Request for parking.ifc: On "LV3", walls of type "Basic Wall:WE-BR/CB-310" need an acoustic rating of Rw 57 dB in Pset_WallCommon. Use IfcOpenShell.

First a look at what the model holds.

```python
import ifcopenshell
import ifcopenshell.util.element

model = ifcopenshell.open("parking.ifc")
print(model.schema)
storey = next(s for s in model.by_type("IfcBuildingStorey") if s.Name == "LV3")
walls = [e for e in ifcopenshell.util.element.get_decomposition(storey) if e.is_a("IfcWall")]
seen = {}
for e in walls:
    element_type = ifcopenshell.util.element.get_type(e)
    key = (element_type.Name if element_type != e and element_type else None, ifcopenshell.util.element.get_pset(e, "Pset_WallCommon", "AcousticRating"))
    seen[key] = seen.get(key, 0) + 1
for (name, value), count in sorted(seen.items(), key=str):
    print(count, "x", name, "|", value)
```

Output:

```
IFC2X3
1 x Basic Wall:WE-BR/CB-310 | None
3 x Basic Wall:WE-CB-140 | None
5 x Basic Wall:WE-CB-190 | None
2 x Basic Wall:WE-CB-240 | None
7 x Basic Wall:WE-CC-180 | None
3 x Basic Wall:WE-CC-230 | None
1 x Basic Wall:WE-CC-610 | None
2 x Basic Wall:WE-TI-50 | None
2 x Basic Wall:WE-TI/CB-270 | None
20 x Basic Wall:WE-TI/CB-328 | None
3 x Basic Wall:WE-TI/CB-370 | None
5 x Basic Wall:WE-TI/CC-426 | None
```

```python
import ifcopenshell
import ifcopenshell.api.pset
import ifcopenshell.util.element

model = ifcopenshell.open("parking.ifc")

storey = next(s for s in model.by_type("IfcBuildingStorey") if s.Name == "LV3")
walls = [e for e in ifcopenshell.util.element.get_decomposition(storey) if e.is_a("IfcWall")]

count = 0
for e in walls:
    element_type = ifcopenshell.util.element.get_type(e)
    if element_type in (None, e) or element_type.Name != "Basic Wall:WE-BR/CB-310":
        continue
    # add_pset returns the element's existing set when there is one.
    pset = ifcopenshell.api.pset.add_pset(model, product=e, name="Pset_WallCommon")
    ifcopenshell.api.pset.edit_pset(model, pset=pset, properties={"AcousticRating": "Rw 57 dB"})
    count += 1

print(count, "walls updated")

model.write("parking_v2.ifc")
```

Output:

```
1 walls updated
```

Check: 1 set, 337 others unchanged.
